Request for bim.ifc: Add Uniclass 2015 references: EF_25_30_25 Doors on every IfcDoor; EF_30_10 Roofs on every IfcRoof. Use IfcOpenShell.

First a look at what the model holds.

```python
import ifcopenshell

model = ifcopenshell.open("bim.ifc")
print(model.schema)
print("classifications:", [c.Name for c in model.by_type("IfcClassification")])
for ifc_class in ("IfcDoor", "IfcRoof", "IfcStair", "IfcWall", "IfcWindow"):
    print(ifc_class, len(model.by_type(ifc_class)))
```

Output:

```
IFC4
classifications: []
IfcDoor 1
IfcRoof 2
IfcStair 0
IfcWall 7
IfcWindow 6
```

```python
import ifcopenshell
import ifcopenshell.api.classification

model = ifcopenshell.open("bim.ifc")

system = ifcopenshell.api.classification.add_classification(model, classification="Uniclass 2015")

codes = {
    "IfcDoor": ("EF_25_30_25", "Doors"),
    "IfcRoof": ("EF_30_10", "Roofs"),
}
for ifc_class, (code, name) in codes.items():
    products = model.by_type(ifc_class)
    ifcopenshell.api.classification.add_reference(
        model, products=products, classification=system, identification=code, name=name
    )
    print(code, len(products))

model.write("bim-out.ifc")
```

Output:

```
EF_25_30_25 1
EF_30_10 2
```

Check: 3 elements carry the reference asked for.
